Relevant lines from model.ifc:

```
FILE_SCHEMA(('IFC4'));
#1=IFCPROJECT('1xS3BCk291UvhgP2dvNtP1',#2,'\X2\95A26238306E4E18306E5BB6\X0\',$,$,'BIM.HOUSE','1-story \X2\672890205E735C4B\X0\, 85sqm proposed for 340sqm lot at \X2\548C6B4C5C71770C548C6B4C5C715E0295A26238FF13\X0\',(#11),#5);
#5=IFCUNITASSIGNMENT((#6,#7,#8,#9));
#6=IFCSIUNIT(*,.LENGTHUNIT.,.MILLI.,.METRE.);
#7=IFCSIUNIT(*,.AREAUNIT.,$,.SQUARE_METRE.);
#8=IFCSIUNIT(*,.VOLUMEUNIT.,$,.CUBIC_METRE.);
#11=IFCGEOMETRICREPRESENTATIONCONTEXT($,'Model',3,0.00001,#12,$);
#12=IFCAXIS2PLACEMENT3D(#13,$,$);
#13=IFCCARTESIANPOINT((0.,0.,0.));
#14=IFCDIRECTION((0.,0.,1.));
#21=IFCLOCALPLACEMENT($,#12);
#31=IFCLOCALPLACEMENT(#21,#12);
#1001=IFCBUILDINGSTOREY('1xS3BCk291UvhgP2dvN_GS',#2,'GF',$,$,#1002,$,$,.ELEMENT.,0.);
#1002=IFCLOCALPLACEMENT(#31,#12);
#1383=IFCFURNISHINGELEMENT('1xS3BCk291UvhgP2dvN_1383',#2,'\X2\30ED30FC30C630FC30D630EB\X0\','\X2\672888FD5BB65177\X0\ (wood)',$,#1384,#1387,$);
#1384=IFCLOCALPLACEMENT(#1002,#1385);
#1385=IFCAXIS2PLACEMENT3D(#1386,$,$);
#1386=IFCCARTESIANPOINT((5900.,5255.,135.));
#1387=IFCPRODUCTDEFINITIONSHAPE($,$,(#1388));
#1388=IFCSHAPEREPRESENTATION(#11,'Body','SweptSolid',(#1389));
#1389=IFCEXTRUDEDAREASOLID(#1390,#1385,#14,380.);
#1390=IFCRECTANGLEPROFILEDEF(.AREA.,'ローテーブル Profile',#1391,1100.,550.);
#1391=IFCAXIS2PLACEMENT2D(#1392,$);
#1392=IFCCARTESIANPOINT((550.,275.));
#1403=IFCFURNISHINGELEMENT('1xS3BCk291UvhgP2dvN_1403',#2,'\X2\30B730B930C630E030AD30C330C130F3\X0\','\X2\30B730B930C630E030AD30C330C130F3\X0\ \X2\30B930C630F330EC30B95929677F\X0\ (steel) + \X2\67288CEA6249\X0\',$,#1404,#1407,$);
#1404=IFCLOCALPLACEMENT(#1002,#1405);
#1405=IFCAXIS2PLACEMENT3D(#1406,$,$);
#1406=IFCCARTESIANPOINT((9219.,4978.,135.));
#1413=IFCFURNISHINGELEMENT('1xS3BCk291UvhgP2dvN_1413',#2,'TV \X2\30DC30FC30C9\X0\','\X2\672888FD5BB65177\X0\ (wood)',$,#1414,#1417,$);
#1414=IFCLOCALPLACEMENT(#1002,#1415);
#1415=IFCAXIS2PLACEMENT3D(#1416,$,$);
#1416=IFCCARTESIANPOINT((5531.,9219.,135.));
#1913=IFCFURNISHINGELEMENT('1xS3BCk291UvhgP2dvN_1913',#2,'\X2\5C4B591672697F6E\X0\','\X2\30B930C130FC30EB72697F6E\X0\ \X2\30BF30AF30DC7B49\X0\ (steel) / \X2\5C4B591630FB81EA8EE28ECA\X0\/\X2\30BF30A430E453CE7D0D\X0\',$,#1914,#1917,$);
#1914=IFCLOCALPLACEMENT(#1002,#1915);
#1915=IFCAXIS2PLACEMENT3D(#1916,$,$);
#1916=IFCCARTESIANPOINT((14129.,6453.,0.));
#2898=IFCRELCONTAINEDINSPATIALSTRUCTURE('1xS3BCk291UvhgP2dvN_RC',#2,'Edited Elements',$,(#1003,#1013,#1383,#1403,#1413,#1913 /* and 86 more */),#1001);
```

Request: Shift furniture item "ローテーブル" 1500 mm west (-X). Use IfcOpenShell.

```python
import ifcopenshell
import ifcopenshell.api.geometry
import ifcopenshell.util.placement
import ifcopenshell.util.unit

model = ifcopenshell.open("model.ifc")
unit_scale = ifcopenshell.util.unit.calculate_unit_scale(model)

item = model.by_id(1383)
matrix = ifcopenshell.util.placement.get_local_placement(item.ObjectPlacement)
matrix[0, 3] -= 1.5 / unit_scale
ifcopenshell.api.geometry.edit_object_placement(model, product=item, matrix=matrix, is_si=False)

print(ifcopenshell.util.placement.get_local_placement(item.ObjectPlacement).round(3) + 0.0)

model.write("model_rev.ifc")
```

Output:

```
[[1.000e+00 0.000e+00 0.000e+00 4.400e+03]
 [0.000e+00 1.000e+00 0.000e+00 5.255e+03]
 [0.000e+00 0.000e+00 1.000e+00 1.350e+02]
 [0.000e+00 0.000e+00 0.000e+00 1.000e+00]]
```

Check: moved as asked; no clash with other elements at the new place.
